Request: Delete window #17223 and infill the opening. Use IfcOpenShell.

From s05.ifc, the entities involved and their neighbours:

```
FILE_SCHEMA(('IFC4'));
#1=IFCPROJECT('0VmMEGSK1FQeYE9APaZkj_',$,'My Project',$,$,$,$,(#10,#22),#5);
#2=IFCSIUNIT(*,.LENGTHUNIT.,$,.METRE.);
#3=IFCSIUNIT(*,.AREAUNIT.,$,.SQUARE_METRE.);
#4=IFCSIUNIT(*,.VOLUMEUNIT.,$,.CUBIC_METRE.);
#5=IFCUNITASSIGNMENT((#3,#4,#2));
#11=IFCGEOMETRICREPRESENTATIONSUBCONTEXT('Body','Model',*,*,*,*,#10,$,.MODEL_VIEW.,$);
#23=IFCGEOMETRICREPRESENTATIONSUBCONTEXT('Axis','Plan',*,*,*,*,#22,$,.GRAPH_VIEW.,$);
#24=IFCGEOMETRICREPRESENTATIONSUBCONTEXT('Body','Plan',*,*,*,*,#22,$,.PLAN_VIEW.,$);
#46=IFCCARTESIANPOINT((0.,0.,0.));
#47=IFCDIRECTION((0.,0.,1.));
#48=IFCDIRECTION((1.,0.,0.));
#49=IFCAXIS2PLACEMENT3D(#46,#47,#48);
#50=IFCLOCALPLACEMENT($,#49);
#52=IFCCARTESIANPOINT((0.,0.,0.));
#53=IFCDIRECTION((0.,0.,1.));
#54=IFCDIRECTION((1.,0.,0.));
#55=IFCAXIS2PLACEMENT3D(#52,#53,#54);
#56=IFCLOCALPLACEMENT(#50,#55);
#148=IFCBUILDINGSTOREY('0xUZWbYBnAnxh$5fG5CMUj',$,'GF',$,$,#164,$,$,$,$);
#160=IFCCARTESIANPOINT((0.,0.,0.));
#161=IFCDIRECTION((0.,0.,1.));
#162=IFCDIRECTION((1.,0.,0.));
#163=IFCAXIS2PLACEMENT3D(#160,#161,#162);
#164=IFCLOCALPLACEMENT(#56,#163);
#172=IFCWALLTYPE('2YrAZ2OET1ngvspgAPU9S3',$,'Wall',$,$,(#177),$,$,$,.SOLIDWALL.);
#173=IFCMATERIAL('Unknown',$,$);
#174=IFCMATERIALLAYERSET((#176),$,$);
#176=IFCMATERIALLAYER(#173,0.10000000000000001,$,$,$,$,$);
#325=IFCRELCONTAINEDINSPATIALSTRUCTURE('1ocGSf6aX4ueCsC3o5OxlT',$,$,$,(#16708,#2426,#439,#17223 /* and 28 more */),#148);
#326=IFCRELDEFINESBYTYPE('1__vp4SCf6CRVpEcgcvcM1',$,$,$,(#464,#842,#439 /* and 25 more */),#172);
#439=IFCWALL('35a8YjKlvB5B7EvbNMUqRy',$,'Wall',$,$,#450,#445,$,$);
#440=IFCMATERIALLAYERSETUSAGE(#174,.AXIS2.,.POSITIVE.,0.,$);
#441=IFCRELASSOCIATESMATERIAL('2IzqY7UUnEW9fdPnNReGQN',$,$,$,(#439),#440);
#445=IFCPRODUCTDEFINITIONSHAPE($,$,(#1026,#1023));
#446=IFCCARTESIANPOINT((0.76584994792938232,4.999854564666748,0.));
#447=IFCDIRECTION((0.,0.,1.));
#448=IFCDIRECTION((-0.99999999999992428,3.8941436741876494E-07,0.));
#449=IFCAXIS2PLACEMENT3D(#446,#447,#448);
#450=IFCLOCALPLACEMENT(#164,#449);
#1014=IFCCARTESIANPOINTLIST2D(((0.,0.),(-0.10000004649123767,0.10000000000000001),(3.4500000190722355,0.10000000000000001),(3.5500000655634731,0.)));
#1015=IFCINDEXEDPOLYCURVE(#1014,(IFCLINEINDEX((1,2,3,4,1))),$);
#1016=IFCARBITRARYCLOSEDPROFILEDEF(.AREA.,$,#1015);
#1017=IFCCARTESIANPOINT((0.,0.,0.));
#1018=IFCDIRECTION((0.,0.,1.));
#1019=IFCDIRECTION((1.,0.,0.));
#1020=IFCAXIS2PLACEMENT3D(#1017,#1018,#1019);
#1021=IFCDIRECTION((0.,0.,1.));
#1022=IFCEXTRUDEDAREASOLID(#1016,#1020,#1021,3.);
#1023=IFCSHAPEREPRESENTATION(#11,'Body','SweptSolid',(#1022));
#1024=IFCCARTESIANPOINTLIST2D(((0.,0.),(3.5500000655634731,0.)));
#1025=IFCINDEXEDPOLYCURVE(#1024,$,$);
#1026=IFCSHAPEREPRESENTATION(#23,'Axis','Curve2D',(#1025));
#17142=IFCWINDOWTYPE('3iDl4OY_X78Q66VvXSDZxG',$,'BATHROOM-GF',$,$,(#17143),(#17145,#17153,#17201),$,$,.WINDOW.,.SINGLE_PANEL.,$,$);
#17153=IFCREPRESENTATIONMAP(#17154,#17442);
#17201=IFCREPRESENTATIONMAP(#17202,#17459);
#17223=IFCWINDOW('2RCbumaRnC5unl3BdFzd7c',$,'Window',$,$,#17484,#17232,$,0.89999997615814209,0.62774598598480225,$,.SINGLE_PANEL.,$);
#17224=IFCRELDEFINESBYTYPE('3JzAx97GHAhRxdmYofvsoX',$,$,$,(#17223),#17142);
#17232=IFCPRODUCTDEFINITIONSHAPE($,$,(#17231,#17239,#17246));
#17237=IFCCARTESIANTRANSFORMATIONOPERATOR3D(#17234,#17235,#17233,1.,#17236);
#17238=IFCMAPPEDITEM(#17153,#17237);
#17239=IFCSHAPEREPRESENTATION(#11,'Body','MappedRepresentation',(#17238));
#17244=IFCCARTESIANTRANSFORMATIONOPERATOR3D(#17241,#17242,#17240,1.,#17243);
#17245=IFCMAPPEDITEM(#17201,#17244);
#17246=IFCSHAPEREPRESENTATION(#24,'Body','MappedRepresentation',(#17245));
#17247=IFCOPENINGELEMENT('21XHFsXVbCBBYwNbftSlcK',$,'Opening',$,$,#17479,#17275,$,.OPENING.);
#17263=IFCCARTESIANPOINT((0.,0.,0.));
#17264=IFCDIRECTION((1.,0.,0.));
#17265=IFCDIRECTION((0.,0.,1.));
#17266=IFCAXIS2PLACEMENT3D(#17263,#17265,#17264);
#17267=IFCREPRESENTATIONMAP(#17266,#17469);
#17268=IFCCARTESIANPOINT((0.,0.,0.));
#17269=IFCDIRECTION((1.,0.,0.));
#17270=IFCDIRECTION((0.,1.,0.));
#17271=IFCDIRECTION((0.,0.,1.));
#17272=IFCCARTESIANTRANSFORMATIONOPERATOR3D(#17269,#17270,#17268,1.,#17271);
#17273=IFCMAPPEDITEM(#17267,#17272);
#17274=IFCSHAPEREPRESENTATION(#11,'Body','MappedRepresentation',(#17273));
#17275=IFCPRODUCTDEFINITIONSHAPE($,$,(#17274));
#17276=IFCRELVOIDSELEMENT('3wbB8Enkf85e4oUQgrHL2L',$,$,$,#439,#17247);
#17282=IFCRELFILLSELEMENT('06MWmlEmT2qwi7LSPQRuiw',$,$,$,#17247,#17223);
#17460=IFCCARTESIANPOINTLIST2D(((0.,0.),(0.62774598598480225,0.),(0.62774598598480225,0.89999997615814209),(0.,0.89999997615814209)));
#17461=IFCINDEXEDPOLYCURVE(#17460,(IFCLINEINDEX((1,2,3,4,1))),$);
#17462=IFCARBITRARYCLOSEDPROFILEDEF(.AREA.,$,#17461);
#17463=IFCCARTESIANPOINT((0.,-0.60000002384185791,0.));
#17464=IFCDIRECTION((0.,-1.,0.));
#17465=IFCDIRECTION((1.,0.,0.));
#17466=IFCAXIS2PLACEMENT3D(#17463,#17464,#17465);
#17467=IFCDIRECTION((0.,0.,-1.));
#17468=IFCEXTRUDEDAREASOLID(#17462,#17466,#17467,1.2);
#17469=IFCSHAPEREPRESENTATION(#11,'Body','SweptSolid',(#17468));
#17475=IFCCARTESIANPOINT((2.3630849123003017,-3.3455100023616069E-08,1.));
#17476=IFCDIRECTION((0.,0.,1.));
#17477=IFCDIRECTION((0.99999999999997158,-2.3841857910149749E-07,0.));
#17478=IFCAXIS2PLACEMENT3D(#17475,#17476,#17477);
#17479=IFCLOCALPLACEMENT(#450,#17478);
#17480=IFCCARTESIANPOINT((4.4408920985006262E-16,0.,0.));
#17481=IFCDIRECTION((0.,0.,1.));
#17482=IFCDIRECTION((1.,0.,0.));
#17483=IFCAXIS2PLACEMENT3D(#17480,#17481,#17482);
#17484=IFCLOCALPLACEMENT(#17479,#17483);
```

```python
import ifcopenshell
import ifcopenshell.api.feature
import ifcopenshell.api.root
import ifcopenshell.geom
import ifcopenshell.util.shape

model = ifcopenshell.open("s05.ifc")
settings = ifcopenshell.geom.settings()


def volume(element):
    """Net volume in cubic metres, openings subtracted."""
    shape = ifcopenshell.geom.create_shape(settings, element)
    return ifcopenshell.util.shape.get_volume(shape.geometry)


window = model.by_guid("2RCbumaRnC5unl3BdFzd7c")
opening = window.FillsVoids[0].RelatingOpeningElement
wall = opening.VoidsElements[0].RelatingBuildingElement
before = volume(wall)

ifcopenshell.api.root.remove_product(model, product=window)
ifcopenshell.api.feature.remove_feature(model, feature=opening)

after = volume(wall)

print(f"wall volume {before:.3f} -> {after:.3f} m3")

model.write("s05_edited.ifc")
```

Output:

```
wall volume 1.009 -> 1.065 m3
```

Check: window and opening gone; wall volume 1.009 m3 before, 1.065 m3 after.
